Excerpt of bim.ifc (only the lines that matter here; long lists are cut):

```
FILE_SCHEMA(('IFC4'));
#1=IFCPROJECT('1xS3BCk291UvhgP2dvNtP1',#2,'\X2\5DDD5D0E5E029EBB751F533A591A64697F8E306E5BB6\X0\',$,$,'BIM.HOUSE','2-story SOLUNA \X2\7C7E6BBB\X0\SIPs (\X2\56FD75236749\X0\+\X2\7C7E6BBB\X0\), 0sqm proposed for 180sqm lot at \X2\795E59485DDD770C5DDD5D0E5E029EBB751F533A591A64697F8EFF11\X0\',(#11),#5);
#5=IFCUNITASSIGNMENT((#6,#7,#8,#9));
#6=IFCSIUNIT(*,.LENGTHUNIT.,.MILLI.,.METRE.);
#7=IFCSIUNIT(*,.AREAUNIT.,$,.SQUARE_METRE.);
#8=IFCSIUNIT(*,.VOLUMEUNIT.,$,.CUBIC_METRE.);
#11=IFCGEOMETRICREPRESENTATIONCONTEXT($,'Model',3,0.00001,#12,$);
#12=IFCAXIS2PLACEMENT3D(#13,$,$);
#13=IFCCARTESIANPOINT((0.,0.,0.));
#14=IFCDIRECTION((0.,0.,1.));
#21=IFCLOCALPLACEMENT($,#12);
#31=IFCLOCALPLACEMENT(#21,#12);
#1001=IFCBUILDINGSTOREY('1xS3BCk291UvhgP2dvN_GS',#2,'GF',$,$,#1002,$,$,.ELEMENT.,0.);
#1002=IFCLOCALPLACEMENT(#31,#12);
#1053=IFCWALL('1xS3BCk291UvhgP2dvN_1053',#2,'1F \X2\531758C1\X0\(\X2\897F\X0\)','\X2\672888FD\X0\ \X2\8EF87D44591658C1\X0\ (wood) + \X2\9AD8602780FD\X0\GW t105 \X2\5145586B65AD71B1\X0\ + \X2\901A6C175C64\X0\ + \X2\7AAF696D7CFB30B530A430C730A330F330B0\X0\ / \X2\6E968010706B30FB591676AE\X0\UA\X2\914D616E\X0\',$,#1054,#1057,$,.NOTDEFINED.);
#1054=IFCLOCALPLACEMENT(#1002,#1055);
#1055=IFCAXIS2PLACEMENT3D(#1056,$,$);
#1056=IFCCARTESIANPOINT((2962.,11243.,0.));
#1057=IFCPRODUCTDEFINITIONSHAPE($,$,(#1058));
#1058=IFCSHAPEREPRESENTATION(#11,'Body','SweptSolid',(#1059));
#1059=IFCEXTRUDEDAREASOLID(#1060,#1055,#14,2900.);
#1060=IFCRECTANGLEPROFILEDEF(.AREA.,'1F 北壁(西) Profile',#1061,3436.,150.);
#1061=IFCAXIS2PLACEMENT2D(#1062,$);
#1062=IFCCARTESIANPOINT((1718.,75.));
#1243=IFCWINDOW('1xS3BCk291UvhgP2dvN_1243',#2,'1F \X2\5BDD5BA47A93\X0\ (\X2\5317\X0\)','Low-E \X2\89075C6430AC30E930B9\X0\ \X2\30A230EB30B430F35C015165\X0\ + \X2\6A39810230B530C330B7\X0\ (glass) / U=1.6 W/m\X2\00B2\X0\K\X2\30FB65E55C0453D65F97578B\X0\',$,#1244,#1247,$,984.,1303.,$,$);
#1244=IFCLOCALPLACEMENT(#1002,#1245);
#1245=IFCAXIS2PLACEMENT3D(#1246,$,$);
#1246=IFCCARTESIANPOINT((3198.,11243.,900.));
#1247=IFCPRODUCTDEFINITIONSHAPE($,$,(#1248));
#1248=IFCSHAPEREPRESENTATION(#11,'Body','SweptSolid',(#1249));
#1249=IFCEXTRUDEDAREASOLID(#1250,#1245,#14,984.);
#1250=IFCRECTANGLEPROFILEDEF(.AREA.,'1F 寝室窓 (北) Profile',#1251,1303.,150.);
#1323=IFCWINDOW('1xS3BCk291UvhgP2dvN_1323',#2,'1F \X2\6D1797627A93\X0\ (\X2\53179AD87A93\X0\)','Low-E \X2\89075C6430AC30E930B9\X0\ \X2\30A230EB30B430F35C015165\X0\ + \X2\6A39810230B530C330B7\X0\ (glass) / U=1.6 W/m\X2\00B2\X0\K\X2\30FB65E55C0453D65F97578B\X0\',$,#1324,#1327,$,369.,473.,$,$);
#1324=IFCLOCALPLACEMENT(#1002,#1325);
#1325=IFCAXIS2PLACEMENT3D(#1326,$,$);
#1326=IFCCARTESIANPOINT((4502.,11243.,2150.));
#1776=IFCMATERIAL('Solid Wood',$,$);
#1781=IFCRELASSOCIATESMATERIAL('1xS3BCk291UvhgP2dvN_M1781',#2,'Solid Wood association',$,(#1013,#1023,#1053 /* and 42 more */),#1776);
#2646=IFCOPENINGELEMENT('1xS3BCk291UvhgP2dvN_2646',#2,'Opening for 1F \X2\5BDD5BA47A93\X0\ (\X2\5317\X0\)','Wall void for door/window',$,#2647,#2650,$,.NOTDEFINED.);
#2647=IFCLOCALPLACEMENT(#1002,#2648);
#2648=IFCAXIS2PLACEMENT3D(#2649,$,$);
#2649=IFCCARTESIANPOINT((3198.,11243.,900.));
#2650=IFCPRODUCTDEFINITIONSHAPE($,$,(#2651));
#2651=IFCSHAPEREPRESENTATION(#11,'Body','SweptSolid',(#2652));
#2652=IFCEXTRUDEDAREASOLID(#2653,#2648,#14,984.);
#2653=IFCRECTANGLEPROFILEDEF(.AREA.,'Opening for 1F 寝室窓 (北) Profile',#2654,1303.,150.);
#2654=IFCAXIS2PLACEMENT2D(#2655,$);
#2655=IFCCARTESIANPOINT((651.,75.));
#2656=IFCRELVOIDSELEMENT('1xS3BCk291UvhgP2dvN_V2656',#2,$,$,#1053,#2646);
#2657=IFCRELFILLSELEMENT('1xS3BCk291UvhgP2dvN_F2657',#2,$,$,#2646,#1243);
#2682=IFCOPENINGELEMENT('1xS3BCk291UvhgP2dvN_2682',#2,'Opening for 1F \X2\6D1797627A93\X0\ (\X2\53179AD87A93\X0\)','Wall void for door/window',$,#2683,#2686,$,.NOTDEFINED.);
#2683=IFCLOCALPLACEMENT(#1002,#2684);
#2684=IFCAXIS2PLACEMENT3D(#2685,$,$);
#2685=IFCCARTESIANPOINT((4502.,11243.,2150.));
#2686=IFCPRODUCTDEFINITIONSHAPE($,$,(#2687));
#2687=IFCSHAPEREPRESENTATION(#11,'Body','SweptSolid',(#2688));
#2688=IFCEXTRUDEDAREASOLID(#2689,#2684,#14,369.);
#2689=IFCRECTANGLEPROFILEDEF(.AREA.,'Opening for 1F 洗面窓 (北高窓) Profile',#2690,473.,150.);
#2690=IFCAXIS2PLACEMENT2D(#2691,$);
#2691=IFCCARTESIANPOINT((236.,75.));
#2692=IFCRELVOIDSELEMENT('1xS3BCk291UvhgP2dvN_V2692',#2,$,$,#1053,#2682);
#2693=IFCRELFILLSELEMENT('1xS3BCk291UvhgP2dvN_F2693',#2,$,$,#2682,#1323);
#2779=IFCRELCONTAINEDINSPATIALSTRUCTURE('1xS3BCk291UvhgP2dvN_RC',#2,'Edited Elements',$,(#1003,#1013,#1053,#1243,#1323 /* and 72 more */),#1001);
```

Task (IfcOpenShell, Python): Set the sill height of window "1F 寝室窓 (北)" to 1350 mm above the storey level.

```python
import numpy as np
import ifcopenshell
import ifcopenshell.api.geometry
import ifcopenshell.geom
import ifcopenshell.util.element
import ifcopenshell.util.placement
import ifcopenshell.util.shape
import ifcopenshell.util.unit

model = ifcopenshell.open("bim.ifc")
unit_scale = ifcopenshell.util.unit.calculate_unit_scale(model)

window = model.by_guid("1xS3BCk291UvhgP2dvN_1243")
opening = window.FillsVoids[0].RelatingOpeningElement
storey = ifcopenshell.util.element.get_container(window, ifc_class="IfcBuildingStorey")
level = ifcopenshell.util.placement.get_local_placement(storey.ObjectPlacement)[2, 3]

# The opening's origin need not be at the sill, so measure its lowest point.
shape = ifcopenshell.geom.create_shape(ifcopenshell.geom.settings(), opening)
bottom = ifcopenshell.util.shape.get_shape_bottom_elevation(shape, shape.geometry) / unit_scale
dz = level + 1.35 / unit_scale - bottom

shift = np.array([0.0, 0.0, dz])
# The window is not placed relative to its opening, so move both.
for product in (opening, window):
    matrix = ifcopenshell.util.placement.get_local_placement(product.ObjectPlacement)
    matrix[:3, 3] += shift
    ifcopenshell.api.geometry.edit_object_placement(model, product=product, matrix=matrix, is_si=False)

print(f"moved by {dz * unit_scale:+.3f} m")

model.write("bim_edited.ifc")
```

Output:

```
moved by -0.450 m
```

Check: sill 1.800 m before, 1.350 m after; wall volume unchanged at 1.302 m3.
